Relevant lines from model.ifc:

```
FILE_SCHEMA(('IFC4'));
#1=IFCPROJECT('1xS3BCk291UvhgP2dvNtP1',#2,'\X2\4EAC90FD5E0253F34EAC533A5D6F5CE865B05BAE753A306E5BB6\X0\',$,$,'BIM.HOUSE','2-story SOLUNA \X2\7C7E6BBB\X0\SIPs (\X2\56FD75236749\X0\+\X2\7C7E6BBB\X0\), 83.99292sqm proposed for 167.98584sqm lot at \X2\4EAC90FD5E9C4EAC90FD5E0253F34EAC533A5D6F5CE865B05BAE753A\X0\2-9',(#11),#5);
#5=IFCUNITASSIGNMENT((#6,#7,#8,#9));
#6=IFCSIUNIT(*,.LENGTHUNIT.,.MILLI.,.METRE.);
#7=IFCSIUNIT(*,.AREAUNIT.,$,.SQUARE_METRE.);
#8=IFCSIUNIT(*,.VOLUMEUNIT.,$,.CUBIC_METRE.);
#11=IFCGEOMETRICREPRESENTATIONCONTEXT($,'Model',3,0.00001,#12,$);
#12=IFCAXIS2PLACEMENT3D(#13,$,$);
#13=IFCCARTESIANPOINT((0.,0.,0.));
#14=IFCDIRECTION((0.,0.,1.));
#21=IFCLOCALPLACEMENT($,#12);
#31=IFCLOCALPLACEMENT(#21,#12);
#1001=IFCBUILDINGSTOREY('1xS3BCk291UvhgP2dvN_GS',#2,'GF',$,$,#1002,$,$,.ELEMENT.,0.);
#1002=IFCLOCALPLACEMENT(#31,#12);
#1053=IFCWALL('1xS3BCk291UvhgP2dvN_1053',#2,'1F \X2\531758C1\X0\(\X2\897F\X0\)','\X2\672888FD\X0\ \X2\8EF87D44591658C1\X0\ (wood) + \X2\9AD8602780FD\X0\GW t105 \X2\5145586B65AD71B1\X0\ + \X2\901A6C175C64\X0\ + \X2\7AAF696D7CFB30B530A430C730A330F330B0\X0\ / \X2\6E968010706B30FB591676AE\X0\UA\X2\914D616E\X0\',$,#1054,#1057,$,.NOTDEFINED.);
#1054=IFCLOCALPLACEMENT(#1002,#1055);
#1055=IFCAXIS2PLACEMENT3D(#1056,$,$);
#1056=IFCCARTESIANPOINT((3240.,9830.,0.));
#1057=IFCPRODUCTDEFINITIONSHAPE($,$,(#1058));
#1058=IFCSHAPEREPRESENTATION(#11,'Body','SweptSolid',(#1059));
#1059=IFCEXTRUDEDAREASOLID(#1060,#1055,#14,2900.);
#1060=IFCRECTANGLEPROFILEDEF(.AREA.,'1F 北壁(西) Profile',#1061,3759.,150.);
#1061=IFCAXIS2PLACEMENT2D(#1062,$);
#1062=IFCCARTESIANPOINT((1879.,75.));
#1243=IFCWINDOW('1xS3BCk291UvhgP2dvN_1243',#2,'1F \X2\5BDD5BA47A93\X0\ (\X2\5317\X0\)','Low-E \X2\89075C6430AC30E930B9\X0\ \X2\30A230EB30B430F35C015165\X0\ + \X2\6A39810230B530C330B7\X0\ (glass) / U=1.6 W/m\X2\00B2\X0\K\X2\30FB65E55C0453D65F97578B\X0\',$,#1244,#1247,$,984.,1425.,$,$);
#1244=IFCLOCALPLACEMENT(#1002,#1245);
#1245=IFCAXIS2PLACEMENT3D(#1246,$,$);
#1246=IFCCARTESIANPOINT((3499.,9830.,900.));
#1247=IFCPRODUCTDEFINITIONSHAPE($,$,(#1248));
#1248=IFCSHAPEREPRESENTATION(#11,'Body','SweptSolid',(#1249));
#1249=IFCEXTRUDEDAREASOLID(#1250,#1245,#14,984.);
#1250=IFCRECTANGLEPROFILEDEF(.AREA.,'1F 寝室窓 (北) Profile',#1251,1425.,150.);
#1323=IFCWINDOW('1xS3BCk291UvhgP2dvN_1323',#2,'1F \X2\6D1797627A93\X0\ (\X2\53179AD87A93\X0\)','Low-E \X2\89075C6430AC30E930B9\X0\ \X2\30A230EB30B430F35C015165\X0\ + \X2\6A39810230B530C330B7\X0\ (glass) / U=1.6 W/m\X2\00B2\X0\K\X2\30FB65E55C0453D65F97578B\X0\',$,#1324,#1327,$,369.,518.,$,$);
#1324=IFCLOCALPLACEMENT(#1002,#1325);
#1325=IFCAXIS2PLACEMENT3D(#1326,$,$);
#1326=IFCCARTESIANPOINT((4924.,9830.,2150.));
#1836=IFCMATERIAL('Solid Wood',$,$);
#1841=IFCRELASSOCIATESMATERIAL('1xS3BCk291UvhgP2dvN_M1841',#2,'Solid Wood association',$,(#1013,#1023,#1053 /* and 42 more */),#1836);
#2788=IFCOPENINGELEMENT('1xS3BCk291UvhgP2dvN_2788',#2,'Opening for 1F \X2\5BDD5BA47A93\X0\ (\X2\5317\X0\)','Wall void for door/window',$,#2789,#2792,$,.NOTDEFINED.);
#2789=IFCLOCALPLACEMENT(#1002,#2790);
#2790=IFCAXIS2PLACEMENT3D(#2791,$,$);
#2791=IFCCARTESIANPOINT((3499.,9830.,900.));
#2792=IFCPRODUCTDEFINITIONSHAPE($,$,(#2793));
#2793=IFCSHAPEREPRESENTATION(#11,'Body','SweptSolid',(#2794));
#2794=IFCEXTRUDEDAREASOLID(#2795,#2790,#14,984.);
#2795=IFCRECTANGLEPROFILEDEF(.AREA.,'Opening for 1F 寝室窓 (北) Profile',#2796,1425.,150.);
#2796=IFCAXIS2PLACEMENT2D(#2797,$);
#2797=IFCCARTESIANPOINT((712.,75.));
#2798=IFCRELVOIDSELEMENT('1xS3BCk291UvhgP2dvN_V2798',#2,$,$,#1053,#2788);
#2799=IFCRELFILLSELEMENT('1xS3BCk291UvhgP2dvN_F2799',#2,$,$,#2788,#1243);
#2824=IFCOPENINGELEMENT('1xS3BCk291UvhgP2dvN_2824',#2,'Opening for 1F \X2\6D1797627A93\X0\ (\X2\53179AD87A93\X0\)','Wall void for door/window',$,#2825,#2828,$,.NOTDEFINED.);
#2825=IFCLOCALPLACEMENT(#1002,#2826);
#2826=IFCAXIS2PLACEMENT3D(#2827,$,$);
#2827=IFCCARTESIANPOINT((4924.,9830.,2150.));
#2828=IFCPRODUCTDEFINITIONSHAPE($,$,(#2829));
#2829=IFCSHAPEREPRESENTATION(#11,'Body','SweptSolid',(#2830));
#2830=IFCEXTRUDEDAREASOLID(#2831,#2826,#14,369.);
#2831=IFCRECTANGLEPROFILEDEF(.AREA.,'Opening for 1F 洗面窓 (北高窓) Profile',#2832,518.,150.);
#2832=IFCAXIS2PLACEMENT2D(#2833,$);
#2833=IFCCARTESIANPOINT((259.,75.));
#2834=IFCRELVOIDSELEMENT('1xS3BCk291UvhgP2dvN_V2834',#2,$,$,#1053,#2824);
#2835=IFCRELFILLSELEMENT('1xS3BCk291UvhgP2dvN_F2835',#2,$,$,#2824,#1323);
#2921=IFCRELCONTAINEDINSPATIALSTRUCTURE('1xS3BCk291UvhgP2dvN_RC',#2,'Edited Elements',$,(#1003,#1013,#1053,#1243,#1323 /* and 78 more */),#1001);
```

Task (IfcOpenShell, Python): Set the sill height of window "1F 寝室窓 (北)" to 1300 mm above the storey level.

```python
import numpy as np
import ifcopenshell
import ifcopenshell.api.geometry
import ifcopenshell.geom
import ifcopenshell.util.element
import ifcopenshell.util.placement
import ifcopenshell.util.shape
import ifcopenshell.util.unit

model = ifcopenshell.open("model.ifc")
unit_scale = ifcopenshell.util.unit.calculate_unit_scale(model)

window = model.by_guid("1xS3BCk291UvhgP2dvN_1243")
opening = window.FillsVoids[0].RelatingOpeningElement
storey = ifcopenshell.util.element.get_container(window, ifc_class="IfcBuildingStorey")
level = ifcopenshell.util.placement.get_local_placement(storey.ObjectPlacement)[2, 3]

# The opening's origin need not be at the sill, so measure its lowest point.
shape = ifcopenshell.geom.create_shape(ifcopenshell.geom.settings(), opening)
bottom = ifcopenshell.util.shape.get_shape_bottom_elevation(shape, shape.geometry) / unit_scale
dz = level + 1.3 / unit_scale - bottom

shift = np.array([0.0, 0.0, dz])
# The window is not placed relative to its opening, so move both.
for product in (opening, window):
    matrix = ifcopenshell.util.placement.get_local_placement(product.ObjectPlacement)
    matrix[:3, 3] += shift
    ifcopenshell.api.geometry.edit_object_placement(model, product=product, matrix=matrix, is_si=False)

print(f"moved by {dz * unit_scale:+.3f} m")

model.write("model_edited.ifc")
```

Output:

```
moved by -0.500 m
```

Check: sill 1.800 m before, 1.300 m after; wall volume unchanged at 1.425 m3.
